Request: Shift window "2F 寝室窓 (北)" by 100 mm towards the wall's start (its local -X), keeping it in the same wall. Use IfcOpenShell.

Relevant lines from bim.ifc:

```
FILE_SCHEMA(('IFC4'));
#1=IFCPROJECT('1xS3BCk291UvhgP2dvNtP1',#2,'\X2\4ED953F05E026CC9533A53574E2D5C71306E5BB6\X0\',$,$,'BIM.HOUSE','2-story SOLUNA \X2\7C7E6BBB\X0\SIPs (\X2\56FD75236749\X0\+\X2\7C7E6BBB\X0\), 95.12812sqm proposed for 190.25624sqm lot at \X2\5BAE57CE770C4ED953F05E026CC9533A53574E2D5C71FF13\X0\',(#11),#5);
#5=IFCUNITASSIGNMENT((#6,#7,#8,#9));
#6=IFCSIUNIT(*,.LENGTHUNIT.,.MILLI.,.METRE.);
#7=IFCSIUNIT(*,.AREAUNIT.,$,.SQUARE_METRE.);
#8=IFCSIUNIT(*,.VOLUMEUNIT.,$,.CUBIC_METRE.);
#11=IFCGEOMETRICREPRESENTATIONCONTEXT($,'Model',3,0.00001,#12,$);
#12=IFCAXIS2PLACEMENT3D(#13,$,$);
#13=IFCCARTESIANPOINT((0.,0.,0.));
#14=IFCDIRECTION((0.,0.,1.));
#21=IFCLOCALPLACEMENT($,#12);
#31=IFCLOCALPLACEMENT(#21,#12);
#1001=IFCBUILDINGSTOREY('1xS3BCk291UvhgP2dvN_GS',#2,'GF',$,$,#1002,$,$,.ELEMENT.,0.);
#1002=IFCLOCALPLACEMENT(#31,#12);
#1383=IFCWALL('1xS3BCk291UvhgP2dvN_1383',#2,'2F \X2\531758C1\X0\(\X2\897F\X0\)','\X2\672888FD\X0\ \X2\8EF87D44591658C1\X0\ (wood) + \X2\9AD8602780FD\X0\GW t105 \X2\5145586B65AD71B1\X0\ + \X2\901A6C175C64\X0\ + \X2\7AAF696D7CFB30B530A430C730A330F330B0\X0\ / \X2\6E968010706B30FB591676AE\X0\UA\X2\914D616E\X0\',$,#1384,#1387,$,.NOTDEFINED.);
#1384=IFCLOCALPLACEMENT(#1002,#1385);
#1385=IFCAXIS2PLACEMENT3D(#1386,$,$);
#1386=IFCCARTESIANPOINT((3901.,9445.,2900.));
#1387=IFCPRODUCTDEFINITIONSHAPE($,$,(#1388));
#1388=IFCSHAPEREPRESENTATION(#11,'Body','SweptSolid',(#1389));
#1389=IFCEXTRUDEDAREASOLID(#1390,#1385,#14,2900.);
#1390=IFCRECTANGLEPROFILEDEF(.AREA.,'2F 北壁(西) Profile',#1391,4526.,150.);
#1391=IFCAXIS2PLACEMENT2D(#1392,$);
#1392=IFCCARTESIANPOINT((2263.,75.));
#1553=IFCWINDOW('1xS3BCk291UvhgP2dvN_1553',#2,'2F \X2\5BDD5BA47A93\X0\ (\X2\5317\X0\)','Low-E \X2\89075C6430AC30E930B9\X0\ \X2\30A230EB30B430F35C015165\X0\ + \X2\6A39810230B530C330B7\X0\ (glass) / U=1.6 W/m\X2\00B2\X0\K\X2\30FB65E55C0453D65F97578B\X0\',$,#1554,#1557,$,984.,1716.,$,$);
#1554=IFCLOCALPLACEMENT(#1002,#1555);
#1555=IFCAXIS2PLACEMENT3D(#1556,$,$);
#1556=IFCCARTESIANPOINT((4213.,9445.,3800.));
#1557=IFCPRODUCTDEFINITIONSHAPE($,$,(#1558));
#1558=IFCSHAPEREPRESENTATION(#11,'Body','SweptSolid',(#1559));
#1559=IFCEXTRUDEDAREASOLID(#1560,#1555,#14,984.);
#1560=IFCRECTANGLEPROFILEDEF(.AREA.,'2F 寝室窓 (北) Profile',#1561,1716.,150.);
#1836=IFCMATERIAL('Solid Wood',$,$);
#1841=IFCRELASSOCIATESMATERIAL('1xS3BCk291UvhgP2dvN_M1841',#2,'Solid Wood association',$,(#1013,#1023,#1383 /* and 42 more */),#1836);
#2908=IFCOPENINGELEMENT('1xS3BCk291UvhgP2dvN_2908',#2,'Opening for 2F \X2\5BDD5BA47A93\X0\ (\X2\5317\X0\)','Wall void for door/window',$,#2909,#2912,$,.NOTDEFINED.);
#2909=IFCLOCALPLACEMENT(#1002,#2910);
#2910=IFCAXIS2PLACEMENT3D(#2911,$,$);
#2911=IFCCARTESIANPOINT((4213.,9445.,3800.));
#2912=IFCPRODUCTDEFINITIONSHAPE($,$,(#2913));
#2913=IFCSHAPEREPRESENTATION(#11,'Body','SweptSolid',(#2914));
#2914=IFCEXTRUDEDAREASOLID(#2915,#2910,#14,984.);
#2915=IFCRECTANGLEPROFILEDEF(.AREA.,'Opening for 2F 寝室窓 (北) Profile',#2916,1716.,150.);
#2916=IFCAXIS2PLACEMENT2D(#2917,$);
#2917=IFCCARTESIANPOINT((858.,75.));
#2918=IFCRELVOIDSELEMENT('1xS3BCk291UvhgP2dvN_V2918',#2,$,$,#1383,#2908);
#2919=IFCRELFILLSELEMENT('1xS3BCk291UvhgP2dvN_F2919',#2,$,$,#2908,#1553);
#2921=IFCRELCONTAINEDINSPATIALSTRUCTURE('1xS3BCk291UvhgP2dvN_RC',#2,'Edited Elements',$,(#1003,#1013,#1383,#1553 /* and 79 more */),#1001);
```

```python
import ifcopenshell
import ifcopenshell.api.geometry
import ifcopenshell.util.placement
import ifcopenshell.util.unit

model = ifcopenshell.open("bim.ifc")
unit_scale = ifcopenshell.util.unit.calculate_unit_scale(model)

window = model.by_guid("1xS3BCk291UvhgP2dvN_1553")
opening = window.FillsVoids[0].RelatingOpeningElement
wall = opening.VoidsElements[0].RelatingBuildingElement

wall_matrix = ifcopenshell.util.placement.get_local_placement(wall.ObjectPlacement)
shift = wall_matrix[:3, 0] * -0.1 / unit_scale
before = ifcopenshell.util.placement.get_local_placement(window.ObjectPlacement)[:3, 3].copy()

# The window is not placed relative to its opening, so move both.
for product in (opening, window):
    matrix = ifcopenshell.util.placement.get_local_placement(product.ObjectPlacement)
    matrix[:3, 3] += shift
    ifcopenshell.api.geometry.edit_object_placement(model, product=product, matrix=matrix, is_si=False)

after = ifcopenshell.util.placement.get_local_placement(window.ObjectPlacement)[:3, 3]
print("window moved by", (after - before).round(3) + 0.0)

model.write("bim-out.ifc")
```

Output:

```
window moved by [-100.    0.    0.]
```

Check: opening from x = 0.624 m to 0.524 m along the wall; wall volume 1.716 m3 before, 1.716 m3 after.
